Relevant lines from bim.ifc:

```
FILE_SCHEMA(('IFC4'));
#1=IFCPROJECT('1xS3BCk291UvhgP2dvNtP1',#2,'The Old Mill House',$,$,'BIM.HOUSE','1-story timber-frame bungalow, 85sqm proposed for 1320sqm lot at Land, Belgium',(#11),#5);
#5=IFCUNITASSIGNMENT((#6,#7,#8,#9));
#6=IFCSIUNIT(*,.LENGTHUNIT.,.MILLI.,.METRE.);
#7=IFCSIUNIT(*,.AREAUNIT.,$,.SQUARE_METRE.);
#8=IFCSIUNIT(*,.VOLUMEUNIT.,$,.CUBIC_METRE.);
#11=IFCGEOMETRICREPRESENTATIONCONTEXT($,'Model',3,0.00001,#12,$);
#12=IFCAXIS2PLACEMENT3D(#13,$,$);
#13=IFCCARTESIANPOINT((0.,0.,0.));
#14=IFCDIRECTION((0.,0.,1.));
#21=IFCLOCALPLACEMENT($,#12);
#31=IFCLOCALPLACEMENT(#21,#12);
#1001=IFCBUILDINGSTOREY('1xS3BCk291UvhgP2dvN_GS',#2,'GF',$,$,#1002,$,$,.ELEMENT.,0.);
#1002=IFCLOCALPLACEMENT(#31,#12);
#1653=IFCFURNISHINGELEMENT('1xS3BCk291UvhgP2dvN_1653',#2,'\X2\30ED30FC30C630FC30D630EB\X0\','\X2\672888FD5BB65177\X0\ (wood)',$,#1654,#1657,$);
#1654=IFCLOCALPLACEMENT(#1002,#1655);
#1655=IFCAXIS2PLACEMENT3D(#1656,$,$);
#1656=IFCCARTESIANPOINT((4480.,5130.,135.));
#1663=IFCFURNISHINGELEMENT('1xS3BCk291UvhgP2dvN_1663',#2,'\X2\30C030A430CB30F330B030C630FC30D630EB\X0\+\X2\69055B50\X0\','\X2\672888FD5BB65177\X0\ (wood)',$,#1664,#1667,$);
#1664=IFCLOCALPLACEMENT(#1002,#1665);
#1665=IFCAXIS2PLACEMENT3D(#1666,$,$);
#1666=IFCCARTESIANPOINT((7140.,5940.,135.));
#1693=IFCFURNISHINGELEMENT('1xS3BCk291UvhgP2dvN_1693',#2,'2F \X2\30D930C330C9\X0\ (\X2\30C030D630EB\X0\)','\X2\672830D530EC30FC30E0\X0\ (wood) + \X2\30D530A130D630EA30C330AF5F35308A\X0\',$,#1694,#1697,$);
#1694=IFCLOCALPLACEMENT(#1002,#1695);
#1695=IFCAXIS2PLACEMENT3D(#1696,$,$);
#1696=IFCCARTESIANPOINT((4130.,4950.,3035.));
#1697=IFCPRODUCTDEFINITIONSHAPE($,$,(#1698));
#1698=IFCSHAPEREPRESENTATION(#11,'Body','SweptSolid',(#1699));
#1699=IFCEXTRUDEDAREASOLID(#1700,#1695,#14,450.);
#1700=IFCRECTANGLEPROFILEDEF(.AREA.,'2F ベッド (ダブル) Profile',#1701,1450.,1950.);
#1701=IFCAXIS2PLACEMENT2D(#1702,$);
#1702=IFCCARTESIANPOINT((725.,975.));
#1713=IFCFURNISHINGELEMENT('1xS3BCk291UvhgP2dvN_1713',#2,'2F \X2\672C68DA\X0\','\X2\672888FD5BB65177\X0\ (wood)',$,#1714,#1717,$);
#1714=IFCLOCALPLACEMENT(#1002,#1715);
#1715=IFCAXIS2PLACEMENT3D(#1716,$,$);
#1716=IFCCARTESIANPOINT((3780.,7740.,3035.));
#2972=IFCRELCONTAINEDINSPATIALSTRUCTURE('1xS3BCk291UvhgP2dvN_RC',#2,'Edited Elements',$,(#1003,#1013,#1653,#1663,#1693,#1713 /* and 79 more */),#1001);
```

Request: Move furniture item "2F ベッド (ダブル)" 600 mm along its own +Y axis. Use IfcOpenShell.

```python
import ifcopenshell
import ifcopenshell.api.geometry
import ifcopenshell.util.placement

model = ifcopenshell.open("bim.ifc")

item = model.by_id(1693)
matrix = ifcopenshell.util.placement.get_local_placement(item.ObjectPlacement)
matrix[:3, 3] += matrix[:3, 1] * 600.0
ifcopenshell.api.geometry.edit_object_placement(model, product=item, matrix=matrix, is_si=False)

print(ifcopenshell.util.placement.get_local_placement(item.ObjectPlacement).round(3) + 0.0)

model.write("bim_updated.ifc")
```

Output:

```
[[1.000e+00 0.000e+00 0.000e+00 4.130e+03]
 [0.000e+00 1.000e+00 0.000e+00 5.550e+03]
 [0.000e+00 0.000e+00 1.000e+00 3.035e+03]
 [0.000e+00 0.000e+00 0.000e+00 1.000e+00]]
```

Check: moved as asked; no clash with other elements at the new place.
